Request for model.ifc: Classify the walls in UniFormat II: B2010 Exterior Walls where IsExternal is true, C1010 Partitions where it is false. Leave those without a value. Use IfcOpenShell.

First a look at what the model holds.

```python
import ifcopenshell
import ifcopenshell.util.element

model = ifcopenshell.open("model.ifc")
print(model.schema)
print("classifications:", [c.Name for c in model.by_type("IfcClassification")])
values = [ifcopenshell.util.element.get_pset(e, "Pset_WallCommon", "IsExternal") for e in model.by_type("IfcWall")]
for value in (True, False, None):
    print("IsExternal", value, values.count(value))
```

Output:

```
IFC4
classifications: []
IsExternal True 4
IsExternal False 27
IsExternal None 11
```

```python
import ifcopenshell
import ifcopenshell.api.classification
import ifcopenshell.util.element

model = ifcopenshell.open("model.ifc")

system = ifcopenshell.api.classification.add_classification(model, classification="UniFormat II")

walls = model.by_type("IfcWall")
external = {e: ifcopenshell.util.element.get_pset(e, "Pset_WallCommon", "IsExternal") for e in walls}
for flag, code, name in ((True, "B2010", "Exterior Walls"), (False, "C1010", "Partitions")):
    products = [e for e in walls if external[e] is flag]
    ifcopenshell.api.classification.add_reference(
        model, products=products, classification=system, identification=code, name=name
    )
    print(code, len(products))

model.write("model_edited.ifc")
```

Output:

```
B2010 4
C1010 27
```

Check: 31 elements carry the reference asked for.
